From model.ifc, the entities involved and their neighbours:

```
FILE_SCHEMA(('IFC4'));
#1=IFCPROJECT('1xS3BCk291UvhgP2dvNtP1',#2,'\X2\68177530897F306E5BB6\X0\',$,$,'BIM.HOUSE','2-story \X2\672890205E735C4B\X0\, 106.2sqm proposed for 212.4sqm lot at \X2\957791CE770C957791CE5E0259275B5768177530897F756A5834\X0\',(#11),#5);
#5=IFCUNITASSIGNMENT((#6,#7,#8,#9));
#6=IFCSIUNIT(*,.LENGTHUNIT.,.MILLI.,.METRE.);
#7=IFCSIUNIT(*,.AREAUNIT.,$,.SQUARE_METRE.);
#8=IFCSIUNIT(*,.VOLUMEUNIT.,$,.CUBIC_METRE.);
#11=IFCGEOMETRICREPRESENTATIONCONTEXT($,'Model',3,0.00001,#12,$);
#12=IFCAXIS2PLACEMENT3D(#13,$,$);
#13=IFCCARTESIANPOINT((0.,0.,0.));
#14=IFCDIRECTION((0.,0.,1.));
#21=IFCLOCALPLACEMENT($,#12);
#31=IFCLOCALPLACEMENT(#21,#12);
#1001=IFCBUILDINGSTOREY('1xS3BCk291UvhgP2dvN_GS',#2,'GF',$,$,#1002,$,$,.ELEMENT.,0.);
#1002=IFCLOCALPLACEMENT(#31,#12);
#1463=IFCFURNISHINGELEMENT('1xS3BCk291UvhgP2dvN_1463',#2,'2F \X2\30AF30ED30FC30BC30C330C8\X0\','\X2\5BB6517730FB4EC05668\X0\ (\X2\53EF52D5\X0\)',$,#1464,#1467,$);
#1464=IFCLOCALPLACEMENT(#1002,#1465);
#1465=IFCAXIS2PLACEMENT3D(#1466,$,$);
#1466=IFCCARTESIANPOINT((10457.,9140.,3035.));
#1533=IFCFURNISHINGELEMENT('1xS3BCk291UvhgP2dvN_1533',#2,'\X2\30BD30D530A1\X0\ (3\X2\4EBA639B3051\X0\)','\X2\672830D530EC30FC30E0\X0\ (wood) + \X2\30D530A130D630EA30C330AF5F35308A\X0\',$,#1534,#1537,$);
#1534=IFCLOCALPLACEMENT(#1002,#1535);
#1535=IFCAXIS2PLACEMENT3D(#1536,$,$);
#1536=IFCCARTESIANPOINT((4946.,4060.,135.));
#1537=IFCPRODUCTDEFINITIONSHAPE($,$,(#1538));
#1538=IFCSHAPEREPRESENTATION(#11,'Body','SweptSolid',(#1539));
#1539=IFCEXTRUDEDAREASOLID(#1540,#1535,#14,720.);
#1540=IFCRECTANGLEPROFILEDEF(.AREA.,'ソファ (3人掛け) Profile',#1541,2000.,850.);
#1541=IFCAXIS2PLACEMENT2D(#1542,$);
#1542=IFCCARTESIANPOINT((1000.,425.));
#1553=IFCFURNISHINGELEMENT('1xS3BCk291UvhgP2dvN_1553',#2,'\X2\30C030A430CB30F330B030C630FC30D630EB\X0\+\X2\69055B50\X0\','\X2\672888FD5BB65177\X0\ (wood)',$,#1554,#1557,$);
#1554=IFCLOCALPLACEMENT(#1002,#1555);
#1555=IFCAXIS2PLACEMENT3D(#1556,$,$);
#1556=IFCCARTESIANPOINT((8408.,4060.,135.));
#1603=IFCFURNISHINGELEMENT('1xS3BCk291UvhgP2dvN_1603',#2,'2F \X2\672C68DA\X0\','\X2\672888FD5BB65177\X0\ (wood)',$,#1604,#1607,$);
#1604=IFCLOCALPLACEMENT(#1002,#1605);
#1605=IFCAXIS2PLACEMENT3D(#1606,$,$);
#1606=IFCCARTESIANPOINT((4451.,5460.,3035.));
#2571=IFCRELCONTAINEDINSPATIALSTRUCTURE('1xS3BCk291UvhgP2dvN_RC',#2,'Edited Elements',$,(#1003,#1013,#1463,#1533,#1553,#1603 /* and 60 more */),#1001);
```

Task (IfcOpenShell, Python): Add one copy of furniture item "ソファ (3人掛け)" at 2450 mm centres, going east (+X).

```python
import numpy as np
import ifcopenshell
import ifcopenshell.api.geometry
import ifcopenshell.api.root
import ifcopenshell.util.element
import ifcopenshell.util.placement
import ifcopenshell.util.unit

model = ifcopenshell.open("model.ifc")
unit_scale = ifcopenshell.util.unit.calculate_unit_scale(model)


def reuse_history(source, copy):
    """copy_class also copies each property set's owner history, people and application; keep the originals."""
    for rel in copy.IsDefinedBy:
        if rel.is_a("IfcRelDefinesByProperties") and (history := rel.RelatingPropertyDefinition.OwnerHistory):
            rel.RelatingPropertyDefinition.OwnerHistory = source.OwnerHistory
            ifcopenshell.util.element.remove_deep2(model, history)


source = model.by_guid("1xS3BCk291UvhgP2dvN_1533")
base = ifcopenshell.util.placement.get_local_placement(source.ObjectPlacement)
step = np.array([1.0, 0.0, 0.0]) * 2.45 / unit_scale

for i in range(1, 2):
    copy = ifcopenshell.api.root.copy_class(model, product=source)
    copy.Representation = ifcopenshell.util.element.copy_deep(
        model, source.Representation, exclude=["IfcGeometricRepresentationContext", "IfcRepresentationMap"]
    )
    reuse_history(source, copy)
    matrix = base.copy()
    matrix[:3, 3] += i * step
    print("added at", matrix[:3, 3].round(3) + 0.0)
    ifcopenshell.api.geometry.edit_object_placement(model, product=copy, matrix=matrix, is_si=False)

model.write("model_edited.ifc")
```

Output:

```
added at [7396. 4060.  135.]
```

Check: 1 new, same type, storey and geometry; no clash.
